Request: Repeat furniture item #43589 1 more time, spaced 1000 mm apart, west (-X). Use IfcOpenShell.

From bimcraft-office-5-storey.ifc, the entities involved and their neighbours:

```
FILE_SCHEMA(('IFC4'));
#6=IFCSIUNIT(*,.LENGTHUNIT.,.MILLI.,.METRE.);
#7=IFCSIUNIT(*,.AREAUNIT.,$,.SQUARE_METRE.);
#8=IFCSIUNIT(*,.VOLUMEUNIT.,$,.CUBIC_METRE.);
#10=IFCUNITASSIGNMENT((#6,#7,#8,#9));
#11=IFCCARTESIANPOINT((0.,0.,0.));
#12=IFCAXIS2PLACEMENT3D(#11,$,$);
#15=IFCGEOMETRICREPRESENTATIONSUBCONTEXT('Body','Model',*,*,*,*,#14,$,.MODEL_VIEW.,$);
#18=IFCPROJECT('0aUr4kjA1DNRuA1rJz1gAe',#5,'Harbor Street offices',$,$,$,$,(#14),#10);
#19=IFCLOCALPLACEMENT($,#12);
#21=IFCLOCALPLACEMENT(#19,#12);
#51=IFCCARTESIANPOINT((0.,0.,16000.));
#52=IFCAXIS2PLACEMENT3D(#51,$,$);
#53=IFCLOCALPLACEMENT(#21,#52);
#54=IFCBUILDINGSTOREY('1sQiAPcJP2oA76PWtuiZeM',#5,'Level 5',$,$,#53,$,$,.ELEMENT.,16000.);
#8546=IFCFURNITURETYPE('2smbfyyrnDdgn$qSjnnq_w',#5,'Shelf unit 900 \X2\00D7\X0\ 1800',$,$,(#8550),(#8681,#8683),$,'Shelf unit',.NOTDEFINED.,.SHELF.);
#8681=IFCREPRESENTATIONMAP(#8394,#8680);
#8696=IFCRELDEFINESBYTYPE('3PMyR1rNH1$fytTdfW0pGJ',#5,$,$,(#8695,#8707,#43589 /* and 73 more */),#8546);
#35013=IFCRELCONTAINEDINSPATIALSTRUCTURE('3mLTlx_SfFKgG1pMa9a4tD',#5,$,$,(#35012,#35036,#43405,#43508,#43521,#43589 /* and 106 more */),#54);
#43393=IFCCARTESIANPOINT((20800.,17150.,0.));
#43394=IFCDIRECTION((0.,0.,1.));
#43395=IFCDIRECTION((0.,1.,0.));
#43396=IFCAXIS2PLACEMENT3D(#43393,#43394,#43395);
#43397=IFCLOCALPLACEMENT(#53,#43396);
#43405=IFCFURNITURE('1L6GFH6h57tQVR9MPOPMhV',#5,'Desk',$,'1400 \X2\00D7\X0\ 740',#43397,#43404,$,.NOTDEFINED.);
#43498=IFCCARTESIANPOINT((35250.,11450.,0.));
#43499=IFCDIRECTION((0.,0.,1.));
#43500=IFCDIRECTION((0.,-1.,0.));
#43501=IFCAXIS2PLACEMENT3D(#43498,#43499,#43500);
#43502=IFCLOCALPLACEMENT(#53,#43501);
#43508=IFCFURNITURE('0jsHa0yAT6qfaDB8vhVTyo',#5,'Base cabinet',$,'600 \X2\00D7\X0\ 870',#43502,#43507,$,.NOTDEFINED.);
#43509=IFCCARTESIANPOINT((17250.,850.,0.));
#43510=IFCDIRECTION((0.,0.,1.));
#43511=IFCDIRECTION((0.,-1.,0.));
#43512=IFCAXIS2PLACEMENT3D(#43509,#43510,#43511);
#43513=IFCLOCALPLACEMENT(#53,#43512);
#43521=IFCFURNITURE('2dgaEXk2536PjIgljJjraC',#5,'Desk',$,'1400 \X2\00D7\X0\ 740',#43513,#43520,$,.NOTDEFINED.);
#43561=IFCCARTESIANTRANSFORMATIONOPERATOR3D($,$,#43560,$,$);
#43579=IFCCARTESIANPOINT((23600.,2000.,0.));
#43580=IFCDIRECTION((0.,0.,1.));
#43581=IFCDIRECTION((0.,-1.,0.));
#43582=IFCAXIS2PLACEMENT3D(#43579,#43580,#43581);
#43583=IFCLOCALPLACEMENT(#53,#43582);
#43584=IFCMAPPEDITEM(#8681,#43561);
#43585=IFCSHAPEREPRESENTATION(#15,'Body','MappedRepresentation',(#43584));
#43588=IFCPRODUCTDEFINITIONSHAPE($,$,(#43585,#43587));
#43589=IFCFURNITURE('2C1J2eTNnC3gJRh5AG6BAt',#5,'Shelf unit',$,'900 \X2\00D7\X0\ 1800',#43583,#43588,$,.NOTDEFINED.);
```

```python
import numpy as np
import ifcopenshell
import ifcopenshell.api.geometry
import ifcopenshell.api.root
import ifcopenshell.util.element
import ifcopenshell.util.placement

model = ifcopenshell.open("bimcraft-office-5-storey.ifc")

source = model.by_id(43589)
base = ifcopenshell.util.placement.get_local_placement(source.ObjectPlacement)
step = np.array([-1.0, 0.0, 0.0]) * 1000.0

for i in range(1, 2):
    copy = ifcopenshell.api.root.copy_class(model, product=source)
    copy.Representation = ifcopenshell.util.element.copy_deep(
        model, source.Representation, exclude=["IfcGeometricRepresentationContext", "IfcRepresentationMap"]
    )
    matrix = base.copy()
    matrix[:3, 3] += i * step
    print("added at", matrix[:3, 3].round(3) + 0.0)
    ifcopenshell.api.geometry.edit_object_placement(model, product=copy, matrix=matrix, is_si=False)

model.write("bimcraft-office-5-storey-out.ifc")
```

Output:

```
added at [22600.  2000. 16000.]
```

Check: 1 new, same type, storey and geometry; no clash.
